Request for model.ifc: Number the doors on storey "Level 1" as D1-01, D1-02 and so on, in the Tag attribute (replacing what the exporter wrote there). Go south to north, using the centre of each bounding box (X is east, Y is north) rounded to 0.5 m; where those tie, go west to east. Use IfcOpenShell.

First a look at what the model holds.

```python
import ifcopenshell
import ifcopenshell.util.element
import ifcopenshell.util.placement

model = ifcopenshell.open("model.ifc")
print(model.schema)
storey = next(s for s in model.by_type("IfcBuildingStorey") if s.Name == "Level 1")
doors = [e for e in ifcopenshell.util.element.get_decomposition(storey) if e.is_a("IfcDoor")]
for e in sorted(doors, key=lambda e: e.id()):
    origin = ifcopenshell.util.placement.get_local_placement(e.ObjectPlacement)[:3, 3]
    print(e.id(), e.Tag, e.Name, origin.round(2) + 0.0, sep=" | ")
```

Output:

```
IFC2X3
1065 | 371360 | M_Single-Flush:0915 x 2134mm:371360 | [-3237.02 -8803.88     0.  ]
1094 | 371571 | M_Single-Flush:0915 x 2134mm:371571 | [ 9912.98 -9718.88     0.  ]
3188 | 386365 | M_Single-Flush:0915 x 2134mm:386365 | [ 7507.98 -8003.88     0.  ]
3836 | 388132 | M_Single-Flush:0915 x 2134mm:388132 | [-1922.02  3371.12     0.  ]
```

```python
import ifcopenshell
import ifcopenshell.geom
import ifcopenshell.util.element
import ifcopenshell.util.shape

model = ifcopenshell.open("model.ifc")
settings = ifcopenshell.geom.settings()
settings.set("use-world-coords", True)


def centre(element):
    shape = ifcopenshell.geom.create_shape(settings, element)
    return ifcopenshell.util.shape.get_bbox_centroid(shape.geometry)


storey = next(s for s in model.by_type("IfcBuildingStorey") if s.Name == "Level 1")
doors = [e for e in ifcopenshell.util.element.get_decomposition(storey) if e.is_a("IfcDoor")]

# Insertion points can sit at a corner or the storey origin, so sort by the geometry (in metres).
centres = {e: centre(e) for e in doors}
doors.sort(key=lambda e: (round(centres[e][1] / 0.5), centres[e][0]))

for i, e in enumerate(doors, start=1):
    number = f"D1-{i:02d}"
    e.Tag = number
    print(e.id(), number)

model.write("model_edited.ifc")
```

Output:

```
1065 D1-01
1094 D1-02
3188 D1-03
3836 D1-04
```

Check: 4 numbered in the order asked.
